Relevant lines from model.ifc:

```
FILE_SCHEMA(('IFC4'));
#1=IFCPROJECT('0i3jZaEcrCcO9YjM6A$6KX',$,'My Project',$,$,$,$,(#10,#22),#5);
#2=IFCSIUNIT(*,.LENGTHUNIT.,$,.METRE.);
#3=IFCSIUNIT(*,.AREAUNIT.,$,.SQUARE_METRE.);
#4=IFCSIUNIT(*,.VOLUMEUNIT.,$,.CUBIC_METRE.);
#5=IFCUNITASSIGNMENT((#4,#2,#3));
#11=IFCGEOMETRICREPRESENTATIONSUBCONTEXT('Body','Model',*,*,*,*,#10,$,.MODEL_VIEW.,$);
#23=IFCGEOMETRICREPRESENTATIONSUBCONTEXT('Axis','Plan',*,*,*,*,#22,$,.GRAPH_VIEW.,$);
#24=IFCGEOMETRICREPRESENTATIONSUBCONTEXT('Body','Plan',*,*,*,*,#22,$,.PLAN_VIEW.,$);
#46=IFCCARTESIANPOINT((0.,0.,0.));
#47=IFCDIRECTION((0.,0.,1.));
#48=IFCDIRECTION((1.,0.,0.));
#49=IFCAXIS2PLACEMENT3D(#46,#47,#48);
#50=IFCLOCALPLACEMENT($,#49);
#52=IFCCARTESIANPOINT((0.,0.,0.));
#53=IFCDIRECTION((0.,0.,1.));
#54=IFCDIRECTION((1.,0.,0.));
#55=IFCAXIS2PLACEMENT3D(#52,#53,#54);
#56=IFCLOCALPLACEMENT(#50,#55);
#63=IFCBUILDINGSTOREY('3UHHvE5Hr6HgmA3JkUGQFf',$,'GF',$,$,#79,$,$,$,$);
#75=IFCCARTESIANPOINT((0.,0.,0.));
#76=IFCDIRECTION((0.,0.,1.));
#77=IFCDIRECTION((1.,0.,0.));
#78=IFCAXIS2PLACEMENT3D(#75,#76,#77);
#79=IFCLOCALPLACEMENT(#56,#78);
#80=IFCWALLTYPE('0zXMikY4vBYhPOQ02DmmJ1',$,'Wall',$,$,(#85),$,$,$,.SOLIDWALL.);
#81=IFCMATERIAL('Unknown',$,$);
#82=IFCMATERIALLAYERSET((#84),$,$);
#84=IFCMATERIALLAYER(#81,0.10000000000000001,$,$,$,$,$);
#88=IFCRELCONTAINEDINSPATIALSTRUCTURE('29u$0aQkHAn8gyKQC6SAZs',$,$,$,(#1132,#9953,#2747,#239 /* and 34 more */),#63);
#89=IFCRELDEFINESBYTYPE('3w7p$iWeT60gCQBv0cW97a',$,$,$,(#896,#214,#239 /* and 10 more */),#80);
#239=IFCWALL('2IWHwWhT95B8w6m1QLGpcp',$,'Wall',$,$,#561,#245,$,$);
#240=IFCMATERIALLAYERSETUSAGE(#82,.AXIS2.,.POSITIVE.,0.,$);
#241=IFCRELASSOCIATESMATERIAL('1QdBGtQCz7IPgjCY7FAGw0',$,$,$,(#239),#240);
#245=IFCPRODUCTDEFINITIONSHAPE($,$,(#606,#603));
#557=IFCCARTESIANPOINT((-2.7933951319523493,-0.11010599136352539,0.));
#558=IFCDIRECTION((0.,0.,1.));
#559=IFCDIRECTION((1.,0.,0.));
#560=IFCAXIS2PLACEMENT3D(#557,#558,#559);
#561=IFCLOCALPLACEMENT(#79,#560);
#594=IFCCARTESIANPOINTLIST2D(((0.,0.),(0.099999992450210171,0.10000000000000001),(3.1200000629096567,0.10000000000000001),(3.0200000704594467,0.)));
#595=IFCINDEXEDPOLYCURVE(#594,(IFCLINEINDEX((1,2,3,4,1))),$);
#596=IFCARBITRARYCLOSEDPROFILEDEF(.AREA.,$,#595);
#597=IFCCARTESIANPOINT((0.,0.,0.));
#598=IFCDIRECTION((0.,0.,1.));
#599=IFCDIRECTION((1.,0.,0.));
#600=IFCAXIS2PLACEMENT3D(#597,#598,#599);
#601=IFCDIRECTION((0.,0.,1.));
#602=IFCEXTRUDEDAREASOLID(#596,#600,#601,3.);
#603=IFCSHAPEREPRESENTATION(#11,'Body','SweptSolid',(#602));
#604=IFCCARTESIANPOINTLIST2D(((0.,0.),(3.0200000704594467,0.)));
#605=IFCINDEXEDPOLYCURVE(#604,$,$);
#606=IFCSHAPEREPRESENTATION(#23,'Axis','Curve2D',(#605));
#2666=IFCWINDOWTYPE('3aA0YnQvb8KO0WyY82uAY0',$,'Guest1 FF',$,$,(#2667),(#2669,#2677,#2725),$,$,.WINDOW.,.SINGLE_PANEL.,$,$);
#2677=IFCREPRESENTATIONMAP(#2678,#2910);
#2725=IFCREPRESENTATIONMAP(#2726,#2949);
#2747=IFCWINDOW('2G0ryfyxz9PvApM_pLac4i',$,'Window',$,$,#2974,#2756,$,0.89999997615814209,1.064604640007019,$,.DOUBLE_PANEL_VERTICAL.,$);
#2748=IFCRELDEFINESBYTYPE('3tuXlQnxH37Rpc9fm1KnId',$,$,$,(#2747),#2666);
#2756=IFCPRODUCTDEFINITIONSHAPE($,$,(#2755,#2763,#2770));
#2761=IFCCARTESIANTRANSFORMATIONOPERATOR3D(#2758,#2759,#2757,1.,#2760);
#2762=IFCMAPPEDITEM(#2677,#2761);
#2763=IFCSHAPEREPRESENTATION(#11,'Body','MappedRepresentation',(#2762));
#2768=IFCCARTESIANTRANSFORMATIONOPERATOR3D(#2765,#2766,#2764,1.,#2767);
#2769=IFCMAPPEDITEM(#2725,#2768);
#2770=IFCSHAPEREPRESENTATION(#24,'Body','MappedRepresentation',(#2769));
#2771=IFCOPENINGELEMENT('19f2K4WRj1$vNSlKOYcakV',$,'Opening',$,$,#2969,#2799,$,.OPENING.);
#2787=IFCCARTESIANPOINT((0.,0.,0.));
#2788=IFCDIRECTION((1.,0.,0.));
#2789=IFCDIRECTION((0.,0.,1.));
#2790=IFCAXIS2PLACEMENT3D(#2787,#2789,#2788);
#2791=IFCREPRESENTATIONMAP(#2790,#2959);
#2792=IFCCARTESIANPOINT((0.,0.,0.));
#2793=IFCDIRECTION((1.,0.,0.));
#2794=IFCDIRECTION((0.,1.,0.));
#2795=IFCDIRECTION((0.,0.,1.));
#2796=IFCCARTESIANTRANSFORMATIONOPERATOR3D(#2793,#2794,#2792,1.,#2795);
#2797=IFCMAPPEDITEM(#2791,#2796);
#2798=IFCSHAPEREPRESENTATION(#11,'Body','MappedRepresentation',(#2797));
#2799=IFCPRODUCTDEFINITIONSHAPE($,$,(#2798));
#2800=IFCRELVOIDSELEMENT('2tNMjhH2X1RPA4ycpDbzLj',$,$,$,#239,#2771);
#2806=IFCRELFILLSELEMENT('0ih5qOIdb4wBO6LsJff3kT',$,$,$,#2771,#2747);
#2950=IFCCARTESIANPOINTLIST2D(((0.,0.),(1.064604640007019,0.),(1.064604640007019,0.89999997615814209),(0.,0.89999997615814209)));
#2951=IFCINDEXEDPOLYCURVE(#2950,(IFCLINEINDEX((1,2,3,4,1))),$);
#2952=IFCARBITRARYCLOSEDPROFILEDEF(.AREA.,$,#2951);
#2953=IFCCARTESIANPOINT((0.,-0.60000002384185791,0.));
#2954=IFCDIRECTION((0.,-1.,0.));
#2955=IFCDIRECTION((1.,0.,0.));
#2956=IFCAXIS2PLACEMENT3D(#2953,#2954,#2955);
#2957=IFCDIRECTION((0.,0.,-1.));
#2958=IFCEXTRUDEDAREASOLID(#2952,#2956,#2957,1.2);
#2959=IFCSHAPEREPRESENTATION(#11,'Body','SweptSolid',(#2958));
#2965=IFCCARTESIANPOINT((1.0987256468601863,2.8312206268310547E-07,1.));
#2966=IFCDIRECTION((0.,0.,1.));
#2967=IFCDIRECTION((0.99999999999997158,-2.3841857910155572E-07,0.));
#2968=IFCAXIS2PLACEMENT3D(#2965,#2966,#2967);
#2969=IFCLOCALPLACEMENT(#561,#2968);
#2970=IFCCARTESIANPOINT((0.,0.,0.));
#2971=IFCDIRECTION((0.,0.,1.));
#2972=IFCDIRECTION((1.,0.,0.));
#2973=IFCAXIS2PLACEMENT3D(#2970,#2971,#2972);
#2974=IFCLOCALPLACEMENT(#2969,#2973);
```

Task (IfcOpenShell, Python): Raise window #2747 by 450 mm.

```python
import numpy as np
import ifcopenshell
import ifcopenshell.api.geometry
import ifcopenshell.util.placement
import ifcopenshell.util.unit

model = ifcopenshell.open("model.ifc")
unit_scale = ifcopenshell.util.unit.calculate_unit_scale(model)

window = model.by_guid("2G0ryfyxz9PvApM_pLac4i")
opening = window.FillsVoids[0].RelatingOpeningElement
dz = 0.45

shift = np.array([0.0, 0.0, dz])
# The window is placed relative to its opening, so it follows when the opening moves.
matrix = ifcopenshell.util.placement.get_local_placement(opening.ObjectPlacement)
matrix[:3, 3] += shift
ifcopenshell.api.geometry.edit_object_placement(
    model, product=opening, matrix=matrix, is_si=False, should_transform_children=True
)

print(f"moved by {dz * unit_scale:+.3f} m")

model.write("model_v2.ifc")
```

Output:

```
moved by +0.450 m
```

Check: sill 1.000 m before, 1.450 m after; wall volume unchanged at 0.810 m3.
